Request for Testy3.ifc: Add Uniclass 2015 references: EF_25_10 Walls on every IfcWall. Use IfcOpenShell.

First a look at what the model holds.

```python
import ifcopenshell

model = ifcopenshell.open("Testy3.ifc")
print(model.schema)
print("classifications:", [c.Name for c in model.by_type("IfcClassification")])
for ifc_class in ("IfcDoor", "IfcRoof", "IfcStair", "IfcWall", "IfcWindow"):
    print(ifc_class, len(model.by_type(ifc_class)))
```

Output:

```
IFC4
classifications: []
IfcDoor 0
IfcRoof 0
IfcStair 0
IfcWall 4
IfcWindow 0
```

```python
import ifcopenshell
import ifcopenshell.api.classification

model = ifcopenshell.open("Testy3.ifc")

system = ifcopenshell.api.classification.add_classification(model, classification="Uniclass 2015")

codes = {
    "IfcWall": ("EF_25_10", "Walls"),
}
for ifc_class, (code, name) in codes.items():
    products = model.by_type(ifc_class)
    ifcopenshell.api.classification.add_reference(
        model, products=products, classification=system, identification=code, name=name
    )
    print(code, len(products))

model.write("Testy3_rev.ifc")
```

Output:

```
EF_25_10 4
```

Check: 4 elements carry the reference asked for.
